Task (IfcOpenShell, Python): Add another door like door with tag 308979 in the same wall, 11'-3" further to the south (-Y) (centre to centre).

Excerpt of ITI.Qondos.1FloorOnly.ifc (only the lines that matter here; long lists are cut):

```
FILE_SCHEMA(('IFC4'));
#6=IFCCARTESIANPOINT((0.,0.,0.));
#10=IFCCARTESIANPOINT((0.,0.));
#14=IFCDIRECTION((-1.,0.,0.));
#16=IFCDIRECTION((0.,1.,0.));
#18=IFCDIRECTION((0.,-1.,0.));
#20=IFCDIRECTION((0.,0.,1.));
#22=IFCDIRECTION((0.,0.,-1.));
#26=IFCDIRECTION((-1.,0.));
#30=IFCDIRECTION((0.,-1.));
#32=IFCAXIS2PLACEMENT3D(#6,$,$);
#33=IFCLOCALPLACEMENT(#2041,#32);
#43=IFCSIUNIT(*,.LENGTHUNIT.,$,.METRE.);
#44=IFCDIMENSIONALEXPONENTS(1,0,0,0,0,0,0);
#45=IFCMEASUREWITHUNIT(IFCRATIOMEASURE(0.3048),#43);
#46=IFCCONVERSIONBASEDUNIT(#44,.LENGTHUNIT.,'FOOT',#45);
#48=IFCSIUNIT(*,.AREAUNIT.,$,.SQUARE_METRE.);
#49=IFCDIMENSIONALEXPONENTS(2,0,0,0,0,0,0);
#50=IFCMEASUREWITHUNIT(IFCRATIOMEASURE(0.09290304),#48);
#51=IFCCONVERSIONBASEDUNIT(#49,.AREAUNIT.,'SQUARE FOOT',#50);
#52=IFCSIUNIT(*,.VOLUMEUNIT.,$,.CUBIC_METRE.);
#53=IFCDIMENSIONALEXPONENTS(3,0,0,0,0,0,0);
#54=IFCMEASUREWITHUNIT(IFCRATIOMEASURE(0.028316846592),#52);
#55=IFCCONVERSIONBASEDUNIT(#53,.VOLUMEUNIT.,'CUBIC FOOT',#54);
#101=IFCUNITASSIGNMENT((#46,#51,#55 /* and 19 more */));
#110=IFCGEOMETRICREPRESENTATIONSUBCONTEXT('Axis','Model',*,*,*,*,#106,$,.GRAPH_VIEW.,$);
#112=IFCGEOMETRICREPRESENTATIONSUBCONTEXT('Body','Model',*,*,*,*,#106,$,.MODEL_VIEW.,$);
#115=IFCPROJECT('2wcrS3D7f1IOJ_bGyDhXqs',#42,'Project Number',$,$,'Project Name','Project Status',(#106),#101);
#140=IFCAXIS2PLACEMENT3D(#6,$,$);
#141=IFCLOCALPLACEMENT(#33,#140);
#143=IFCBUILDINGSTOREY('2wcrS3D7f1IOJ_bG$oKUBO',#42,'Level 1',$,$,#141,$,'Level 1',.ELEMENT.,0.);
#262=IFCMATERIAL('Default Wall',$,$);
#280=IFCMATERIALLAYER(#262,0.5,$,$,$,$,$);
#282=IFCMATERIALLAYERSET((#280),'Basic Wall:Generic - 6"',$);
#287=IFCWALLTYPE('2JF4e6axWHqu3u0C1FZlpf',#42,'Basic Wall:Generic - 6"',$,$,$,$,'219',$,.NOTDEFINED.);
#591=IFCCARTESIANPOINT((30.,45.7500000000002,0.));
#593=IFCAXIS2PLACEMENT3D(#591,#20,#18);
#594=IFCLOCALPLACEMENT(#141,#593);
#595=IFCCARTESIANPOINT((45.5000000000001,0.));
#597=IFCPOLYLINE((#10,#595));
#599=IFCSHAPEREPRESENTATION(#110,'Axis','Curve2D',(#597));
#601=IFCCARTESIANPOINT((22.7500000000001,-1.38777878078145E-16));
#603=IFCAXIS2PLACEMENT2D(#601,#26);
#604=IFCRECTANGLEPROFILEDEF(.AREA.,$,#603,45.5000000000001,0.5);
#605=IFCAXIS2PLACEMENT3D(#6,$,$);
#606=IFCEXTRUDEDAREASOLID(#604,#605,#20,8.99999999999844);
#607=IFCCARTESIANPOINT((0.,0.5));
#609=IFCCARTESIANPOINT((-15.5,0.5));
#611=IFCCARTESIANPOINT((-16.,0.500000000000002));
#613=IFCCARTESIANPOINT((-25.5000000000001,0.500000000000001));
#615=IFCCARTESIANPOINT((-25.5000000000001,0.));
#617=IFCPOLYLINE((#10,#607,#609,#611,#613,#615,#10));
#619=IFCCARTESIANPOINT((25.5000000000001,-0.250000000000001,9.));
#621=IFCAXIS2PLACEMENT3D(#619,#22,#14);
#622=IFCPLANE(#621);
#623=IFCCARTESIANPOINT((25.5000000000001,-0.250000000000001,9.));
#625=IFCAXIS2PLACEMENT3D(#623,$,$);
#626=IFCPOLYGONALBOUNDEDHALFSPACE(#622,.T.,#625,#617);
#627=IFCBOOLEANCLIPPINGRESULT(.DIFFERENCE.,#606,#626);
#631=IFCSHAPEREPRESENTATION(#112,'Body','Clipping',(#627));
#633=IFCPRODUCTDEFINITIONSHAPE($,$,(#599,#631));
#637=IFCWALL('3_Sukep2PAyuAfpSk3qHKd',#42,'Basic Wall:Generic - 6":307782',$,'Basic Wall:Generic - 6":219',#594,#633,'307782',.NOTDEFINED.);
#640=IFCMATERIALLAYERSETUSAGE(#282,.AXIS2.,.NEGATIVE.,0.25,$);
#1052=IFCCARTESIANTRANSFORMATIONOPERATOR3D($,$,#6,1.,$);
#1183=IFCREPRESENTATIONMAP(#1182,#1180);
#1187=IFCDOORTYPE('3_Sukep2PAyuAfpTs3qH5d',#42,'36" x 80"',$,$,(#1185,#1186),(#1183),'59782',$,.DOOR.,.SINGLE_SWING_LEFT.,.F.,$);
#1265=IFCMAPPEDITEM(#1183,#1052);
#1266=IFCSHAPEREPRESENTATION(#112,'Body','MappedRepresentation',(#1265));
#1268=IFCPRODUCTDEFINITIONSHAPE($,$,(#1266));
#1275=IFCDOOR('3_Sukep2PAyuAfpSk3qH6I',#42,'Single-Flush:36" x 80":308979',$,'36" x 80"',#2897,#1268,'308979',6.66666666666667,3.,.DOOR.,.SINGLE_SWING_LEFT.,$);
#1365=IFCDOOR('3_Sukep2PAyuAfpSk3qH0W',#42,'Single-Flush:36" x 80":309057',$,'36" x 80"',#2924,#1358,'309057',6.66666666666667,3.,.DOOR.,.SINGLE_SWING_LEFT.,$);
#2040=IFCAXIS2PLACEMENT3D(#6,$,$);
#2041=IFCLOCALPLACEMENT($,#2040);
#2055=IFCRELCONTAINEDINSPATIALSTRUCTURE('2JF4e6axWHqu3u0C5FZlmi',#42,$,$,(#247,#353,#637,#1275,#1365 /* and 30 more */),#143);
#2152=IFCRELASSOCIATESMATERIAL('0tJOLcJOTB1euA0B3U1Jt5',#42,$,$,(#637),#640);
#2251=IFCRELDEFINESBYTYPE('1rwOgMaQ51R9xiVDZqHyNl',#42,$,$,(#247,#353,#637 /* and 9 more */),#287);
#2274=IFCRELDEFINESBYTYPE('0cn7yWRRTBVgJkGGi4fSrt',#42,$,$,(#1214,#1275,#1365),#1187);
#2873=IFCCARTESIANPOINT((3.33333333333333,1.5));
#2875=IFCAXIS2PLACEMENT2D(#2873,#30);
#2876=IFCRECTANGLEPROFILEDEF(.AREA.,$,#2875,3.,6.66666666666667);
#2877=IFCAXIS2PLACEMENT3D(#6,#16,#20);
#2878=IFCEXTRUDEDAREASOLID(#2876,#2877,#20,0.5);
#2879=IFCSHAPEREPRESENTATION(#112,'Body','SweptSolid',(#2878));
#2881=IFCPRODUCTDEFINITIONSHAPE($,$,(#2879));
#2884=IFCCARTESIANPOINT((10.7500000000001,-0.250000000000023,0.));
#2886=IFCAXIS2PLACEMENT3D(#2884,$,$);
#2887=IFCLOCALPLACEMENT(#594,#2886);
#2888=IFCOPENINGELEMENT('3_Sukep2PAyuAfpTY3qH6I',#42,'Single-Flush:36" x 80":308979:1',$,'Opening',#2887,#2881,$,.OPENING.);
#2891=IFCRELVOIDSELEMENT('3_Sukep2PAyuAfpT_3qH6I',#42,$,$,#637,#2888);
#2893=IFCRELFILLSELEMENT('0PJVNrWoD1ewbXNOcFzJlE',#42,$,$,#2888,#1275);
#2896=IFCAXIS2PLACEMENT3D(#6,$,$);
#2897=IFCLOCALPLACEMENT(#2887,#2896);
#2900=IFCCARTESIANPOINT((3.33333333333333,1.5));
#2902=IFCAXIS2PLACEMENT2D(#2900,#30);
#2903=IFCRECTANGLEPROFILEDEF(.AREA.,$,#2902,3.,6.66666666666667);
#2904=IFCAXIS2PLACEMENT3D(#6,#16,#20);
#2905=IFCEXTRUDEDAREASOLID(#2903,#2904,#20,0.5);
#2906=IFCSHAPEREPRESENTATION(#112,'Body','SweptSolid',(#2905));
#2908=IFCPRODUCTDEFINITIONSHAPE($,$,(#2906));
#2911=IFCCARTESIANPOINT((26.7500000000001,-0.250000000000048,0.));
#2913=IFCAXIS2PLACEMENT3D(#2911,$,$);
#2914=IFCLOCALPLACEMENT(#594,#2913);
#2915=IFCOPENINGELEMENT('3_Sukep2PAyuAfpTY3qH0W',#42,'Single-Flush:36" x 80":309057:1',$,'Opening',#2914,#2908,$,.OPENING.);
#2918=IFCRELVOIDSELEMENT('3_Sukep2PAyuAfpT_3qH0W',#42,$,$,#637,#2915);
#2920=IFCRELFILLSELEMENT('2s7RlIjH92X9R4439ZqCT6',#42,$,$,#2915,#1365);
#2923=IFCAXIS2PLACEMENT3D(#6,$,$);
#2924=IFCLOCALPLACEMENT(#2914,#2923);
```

```python
import ifcopenshell
import ifcopenshell.api.feature
import ifcopenshell.api.geometry
import ifcopenshell.api.root
import ifcopenshell.geom
import ifcopenshell.util.element
import ifcopenshell.util.placement
import ifcopenshell.util.shape
import ifcopenshell.util.unit

model = ifcopenshell.open("ITI.Qondos.1FloorOnly.ifc")
unit_scale = ifcopenshell.util.unit.calculate_unit_scale(model)
settings = ifcopenshell.geom.settings()


def volume(element):
    """Net volume in cubic metres, openings subtracted."""
    shape = ifcopenshell.geom.create_shape(settings, element)
    return ifcopenshell.util.shape.get_volume(shape.geometry)


def reuse_history(source, copy):
    """copy_class also copies each property set's owner history, people and application; keep the originals."""
    for rel in copy.IsDefinedBy:
        if rel.is_a("IfcRelDefinesByProperties") and (history := rel.RelatingPropertyDefinition.OwnerHistory):
            rel.RelatingPropertyDefinition.OwnerHistory = source.OwnerHistory
            ifcopenshell.util.element.remove_deep2(model, history)


door = model.by_id(1275)
opening = door.FillsVoids[0].RelatingOpeningElement
wall = opening.VoidsElements[0].RelatingBuildingElement
before = volume(wall)
shift = ifcopenshell.util.placement.get_local_placement(wall.ObjectPlacement)[:3, 0] * 135 * 0.0254 / unit_scale

# copy_class copies the void relationship, type, container and properties, but no geometry.
new_opening = ifcopenshell.api.root.copy_class(model, product=opening)
new_opening.Representation = ifcopenshell.util.element.copy_deep(
    model, opening.Representation, exclude=["IfcGeometricRepresentationContext", "IfcRepresentationMap"]
)
new_opening.Name = 'Single-Flush:36" x 80"'
new_door = ifcopenshell.api.root.copy_class(model, product=door)
new_door.Representation = ifcopenshell.util.element.copy_deep(
    model, door.Representation, exclude=["IfcGeometricRepresentationContext", "IfcRepresentationMap"]
)
new_door.Name = 'Single-Flush:36" x 80"'
new_door.Tag = None
reuse_history(door, new_door)
ifcopenshell.api.feature.add_filling(model, opening=new_opening, element=new_door)

for old, new in ((opening, new_opening), (door, new_door)):
    matrix = ifcopenshell.util.placement.get_local_placement(old.ObjectPlacement)
    matrix[:3, 3] += shift
    ifcopenshell.api.geometry.edit_object_placement(model, product=new, matrix=matrix, is_si=False)

after = volume(wall)

print(f"wall volume {before:.3f} -> {after:.3f} m3")

model.write("ITI.Qondos.1FloorOnly_rev.ifc")
```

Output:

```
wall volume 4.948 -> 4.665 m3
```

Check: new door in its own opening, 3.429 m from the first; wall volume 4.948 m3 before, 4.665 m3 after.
